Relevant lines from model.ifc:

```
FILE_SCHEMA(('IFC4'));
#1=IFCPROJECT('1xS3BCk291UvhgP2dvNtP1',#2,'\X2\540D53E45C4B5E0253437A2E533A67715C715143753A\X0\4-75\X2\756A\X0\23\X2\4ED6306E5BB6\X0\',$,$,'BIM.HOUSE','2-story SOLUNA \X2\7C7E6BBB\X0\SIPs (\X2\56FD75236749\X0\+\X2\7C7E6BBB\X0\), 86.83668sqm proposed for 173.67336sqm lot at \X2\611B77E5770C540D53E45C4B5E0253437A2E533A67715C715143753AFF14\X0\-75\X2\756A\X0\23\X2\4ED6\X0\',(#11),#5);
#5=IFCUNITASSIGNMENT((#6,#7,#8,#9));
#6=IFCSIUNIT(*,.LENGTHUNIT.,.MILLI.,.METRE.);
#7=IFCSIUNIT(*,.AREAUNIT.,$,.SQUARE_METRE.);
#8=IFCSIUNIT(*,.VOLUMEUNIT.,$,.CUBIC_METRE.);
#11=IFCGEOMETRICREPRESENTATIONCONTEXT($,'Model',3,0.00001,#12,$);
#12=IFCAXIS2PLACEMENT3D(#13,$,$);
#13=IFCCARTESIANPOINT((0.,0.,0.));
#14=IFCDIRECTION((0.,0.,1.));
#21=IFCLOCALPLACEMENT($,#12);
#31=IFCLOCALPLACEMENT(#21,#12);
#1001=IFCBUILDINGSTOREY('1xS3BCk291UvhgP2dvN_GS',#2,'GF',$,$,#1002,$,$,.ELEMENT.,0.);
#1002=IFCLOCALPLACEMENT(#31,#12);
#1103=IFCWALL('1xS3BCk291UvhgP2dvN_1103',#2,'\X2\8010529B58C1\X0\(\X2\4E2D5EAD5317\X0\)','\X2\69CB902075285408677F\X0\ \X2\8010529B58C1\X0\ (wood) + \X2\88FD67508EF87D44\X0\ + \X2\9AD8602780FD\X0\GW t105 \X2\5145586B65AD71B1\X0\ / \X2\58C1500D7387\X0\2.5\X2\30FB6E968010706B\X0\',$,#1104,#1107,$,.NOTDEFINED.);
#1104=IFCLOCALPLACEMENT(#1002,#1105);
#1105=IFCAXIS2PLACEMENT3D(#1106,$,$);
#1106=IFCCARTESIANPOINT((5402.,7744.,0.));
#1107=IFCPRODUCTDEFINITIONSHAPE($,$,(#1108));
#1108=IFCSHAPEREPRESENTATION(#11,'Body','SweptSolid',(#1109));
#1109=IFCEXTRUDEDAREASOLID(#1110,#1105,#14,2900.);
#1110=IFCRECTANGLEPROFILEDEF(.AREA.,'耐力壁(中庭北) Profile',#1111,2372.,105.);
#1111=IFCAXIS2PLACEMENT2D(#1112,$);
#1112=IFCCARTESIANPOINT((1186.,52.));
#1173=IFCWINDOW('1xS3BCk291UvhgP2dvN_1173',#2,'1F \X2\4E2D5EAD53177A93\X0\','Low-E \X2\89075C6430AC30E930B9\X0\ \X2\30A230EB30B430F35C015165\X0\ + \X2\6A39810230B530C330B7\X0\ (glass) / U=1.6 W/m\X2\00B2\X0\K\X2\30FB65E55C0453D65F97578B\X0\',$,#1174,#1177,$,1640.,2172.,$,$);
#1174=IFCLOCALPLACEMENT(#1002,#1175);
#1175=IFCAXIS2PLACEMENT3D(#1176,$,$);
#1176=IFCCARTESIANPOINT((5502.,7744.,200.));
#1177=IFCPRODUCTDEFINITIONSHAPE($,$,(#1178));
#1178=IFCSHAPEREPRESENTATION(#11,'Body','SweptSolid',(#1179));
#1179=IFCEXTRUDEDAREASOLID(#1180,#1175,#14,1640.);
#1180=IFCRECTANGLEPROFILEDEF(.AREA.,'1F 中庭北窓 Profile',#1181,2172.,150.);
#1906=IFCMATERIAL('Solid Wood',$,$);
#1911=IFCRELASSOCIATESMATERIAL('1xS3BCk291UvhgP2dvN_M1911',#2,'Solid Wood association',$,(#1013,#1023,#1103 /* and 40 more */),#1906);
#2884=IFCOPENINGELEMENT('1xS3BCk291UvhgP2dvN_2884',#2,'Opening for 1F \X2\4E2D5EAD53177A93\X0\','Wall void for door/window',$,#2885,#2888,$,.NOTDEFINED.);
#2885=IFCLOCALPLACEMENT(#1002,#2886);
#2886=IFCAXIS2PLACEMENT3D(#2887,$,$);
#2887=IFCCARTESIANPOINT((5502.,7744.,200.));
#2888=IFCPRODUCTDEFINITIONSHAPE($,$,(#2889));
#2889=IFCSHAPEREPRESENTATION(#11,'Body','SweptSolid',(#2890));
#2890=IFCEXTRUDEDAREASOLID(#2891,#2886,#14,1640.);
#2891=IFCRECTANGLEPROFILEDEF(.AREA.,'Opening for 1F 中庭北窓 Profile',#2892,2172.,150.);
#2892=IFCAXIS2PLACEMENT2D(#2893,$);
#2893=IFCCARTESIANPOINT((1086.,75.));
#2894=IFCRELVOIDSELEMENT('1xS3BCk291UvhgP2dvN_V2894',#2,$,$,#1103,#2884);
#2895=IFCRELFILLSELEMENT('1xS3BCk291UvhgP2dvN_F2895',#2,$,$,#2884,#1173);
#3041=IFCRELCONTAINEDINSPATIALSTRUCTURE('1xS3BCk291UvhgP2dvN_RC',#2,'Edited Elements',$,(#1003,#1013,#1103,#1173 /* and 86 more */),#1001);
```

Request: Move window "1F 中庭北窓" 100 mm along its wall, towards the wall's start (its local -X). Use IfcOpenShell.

```python
import ifcopenshell
import ifcopenshell.api.geometry
import ifcopenshell.util.placement
import ifcopenshell.util.unit

model = ifcopenshell.open("model.ifc")
unit_scale = ifcopenshell.util.unit.calculate_unit_scale(model)

window = model.by_guid("1xS3BCk291UvhgP2dvN_1173")
opening = window.FillsVoids[0].RelatingOpeningElement
wall = opening.VoidsElements[0].RelatingBuildingElement

wall_matrix = ifcopenshell.util.placement.get_local_placement(wall.ObjectPlacement)
shift = wall_matrix[:3, 0] * -0.1 / unit_scale
before = ifcopenshell.util.placement.get_local_placement(window.ObjectPlacement)[:3, 3].copy()

# The window is not placed relative to its opening, so move both.
for product in (opening, window):
    matrix = ifcopenshell.util.placement.get_local_placement(product.ObjectPlacement)
    matrix[:3, 3] += shift
    ifcopenshell.api.geometry.edit_object_placement(model, product=product, matrix=matrix, is_si=False)

after = ifcopenshell.util.placement.get_local_placement(window.ObjectPlacement)[:3, 3]
print("window moved by", (after - before).round(3) + 0.0)

model.write("model_edited.ifc")
```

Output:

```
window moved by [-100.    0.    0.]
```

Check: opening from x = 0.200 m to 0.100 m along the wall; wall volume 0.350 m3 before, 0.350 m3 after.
